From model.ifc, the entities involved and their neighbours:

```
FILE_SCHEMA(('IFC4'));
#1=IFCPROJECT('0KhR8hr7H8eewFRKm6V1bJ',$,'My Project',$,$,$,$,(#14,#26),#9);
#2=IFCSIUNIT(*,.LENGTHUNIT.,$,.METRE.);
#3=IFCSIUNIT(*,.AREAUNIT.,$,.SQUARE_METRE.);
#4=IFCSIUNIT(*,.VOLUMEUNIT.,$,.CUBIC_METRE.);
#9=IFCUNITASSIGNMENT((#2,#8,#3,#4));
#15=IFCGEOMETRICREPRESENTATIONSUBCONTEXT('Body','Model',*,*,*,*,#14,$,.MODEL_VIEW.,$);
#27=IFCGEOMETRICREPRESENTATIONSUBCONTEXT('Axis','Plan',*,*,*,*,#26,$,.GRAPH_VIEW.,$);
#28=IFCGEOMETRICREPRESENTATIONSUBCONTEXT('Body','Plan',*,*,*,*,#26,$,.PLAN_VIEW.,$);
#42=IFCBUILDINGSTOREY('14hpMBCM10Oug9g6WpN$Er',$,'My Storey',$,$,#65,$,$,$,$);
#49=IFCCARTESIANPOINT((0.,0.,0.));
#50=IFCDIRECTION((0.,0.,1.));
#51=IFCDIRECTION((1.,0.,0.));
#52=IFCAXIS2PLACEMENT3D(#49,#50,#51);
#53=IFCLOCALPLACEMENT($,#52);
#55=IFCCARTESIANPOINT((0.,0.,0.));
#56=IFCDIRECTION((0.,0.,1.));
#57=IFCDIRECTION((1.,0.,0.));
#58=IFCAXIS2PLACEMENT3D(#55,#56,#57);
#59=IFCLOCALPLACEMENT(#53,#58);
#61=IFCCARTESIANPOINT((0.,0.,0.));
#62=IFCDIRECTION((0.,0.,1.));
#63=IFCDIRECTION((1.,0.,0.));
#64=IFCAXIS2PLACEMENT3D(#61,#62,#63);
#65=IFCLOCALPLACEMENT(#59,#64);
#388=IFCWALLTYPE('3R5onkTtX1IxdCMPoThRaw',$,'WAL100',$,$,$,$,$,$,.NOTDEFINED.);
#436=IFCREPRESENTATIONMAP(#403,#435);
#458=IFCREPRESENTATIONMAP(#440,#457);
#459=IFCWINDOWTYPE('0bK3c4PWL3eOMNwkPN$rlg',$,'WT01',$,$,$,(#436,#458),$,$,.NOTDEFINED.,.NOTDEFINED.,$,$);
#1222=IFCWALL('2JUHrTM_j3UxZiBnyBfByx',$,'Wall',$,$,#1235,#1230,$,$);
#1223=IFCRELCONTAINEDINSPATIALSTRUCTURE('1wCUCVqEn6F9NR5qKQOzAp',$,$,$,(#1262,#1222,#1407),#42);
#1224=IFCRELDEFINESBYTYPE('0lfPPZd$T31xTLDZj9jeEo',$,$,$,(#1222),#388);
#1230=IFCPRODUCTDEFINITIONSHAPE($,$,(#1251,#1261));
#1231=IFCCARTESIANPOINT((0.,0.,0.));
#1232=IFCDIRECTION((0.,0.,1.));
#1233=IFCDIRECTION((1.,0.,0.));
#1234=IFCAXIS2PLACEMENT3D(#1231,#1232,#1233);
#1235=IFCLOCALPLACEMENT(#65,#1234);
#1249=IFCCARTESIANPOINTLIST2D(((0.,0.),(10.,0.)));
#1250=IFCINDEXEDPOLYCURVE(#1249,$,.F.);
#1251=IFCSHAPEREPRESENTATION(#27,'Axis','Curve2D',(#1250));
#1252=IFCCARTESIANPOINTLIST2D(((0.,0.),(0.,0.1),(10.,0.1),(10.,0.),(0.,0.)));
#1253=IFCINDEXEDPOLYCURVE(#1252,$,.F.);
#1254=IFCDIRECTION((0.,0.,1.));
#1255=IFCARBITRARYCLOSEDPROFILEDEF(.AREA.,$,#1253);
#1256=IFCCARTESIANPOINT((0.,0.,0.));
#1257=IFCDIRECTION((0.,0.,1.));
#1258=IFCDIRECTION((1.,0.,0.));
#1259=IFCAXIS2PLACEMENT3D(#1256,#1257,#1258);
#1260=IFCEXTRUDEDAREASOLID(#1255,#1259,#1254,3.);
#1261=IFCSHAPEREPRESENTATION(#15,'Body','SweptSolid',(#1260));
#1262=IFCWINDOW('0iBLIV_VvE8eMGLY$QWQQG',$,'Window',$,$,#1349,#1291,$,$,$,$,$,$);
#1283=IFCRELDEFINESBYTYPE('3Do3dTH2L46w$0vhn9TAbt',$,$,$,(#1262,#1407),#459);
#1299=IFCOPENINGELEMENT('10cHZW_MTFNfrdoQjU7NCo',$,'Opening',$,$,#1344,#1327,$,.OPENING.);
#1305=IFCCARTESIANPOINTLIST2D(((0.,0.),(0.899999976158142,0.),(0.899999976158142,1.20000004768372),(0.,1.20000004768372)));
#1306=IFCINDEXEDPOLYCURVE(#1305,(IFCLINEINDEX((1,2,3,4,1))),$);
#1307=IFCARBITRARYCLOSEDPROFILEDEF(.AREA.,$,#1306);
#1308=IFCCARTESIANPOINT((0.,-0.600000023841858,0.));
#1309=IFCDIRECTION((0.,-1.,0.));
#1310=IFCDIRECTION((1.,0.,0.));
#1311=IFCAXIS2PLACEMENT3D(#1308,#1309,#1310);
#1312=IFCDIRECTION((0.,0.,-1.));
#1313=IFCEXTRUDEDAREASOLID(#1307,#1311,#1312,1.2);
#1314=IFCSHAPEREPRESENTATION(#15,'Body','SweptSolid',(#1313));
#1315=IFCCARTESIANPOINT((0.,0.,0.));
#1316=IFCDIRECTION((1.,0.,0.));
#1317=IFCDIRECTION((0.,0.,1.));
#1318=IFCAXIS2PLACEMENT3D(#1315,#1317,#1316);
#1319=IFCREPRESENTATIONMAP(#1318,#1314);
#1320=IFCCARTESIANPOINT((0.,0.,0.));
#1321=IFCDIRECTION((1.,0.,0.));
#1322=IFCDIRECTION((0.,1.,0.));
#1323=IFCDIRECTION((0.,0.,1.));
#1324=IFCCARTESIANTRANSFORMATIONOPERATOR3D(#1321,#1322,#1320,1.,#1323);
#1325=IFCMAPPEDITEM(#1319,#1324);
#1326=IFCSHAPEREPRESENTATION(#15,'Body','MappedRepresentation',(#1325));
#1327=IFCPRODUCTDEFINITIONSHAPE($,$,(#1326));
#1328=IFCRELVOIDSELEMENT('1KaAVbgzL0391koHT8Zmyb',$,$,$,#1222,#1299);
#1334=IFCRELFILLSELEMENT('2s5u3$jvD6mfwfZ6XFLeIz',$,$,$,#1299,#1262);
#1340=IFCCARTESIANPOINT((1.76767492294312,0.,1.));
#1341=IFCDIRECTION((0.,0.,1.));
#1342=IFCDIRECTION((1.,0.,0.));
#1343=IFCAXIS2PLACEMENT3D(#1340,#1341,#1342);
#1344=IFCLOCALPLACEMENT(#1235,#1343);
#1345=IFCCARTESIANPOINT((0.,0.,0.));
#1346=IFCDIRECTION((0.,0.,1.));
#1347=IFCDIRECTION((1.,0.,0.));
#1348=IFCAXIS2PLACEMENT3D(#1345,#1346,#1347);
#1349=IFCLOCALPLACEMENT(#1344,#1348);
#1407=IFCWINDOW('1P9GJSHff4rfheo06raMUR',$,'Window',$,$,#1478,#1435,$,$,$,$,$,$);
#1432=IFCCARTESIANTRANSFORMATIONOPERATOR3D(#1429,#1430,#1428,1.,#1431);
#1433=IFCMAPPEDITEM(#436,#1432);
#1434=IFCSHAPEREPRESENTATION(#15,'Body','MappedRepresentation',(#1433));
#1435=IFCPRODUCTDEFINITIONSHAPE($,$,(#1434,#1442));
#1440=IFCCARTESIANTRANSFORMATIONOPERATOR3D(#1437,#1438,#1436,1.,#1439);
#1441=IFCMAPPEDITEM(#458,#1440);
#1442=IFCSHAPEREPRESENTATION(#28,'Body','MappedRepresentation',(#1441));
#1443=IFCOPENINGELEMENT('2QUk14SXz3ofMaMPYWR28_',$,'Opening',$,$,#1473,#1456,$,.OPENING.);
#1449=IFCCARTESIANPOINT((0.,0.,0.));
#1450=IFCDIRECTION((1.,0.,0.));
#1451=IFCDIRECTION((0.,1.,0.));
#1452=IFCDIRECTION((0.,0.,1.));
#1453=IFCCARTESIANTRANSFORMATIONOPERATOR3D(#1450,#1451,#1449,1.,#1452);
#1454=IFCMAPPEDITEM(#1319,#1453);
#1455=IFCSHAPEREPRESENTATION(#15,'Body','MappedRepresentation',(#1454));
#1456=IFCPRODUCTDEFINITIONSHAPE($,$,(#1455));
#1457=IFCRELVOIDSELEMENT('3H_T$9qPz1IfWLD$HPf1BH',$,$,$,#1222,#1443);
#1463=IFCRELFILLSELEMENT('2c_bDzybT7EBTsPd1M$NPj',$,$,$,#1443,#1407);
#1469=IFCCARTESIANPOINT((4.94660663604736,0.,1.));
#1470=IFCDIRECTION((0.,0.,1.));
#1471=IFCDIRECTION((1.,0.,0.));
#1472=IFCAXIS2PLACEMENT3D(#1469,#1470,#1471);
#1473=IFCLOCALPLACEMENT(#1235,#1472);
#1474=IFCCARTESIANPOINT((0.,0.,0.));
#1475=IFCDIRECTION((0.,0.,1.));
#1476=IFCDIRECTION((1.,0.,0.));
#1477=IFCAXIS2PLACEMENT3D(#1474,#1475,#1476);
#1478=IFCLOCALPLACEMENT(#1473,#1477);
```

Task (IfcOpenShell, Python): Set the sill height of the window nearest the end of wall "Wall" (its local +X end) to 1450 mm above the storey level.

```python
import numpy as np
import ifcopenshell
import ifcopenshell.api.geometry
import ifcopenshell.geom
import ifcopenshell.util.element
import ifcopenshell.util.placement
import ifcopenshell.util.shape
import ifcopenshell.util.unit

model = ifcopenshell.open("model.ifc")
unit_scale = ifcopenshell.util.unit.calculate_unit_scale(model)

window = model.by_guid("1P9GJSHff4rfheo06raMUR")
opening = window.FillsVoids[0].RelatingOpeningElement
storey = ifcopenshell.util.element.get_container(window, ifc_class="IfcBuildingStorey")
level = ifcopenshell.util.placement.get_local_placement(storey.ObjectPlacement)[2, 3]

# The opening's origin need not be at the sill, so measure its lowest point.
shape = ifcopenshell.geom.create_shape(ifcopenshell.geom.settings(), opening)
bottom = ifcopenshell.util.shape.get_shape_bottom_elevation(shape, shape.geometry) / unit_scale
dz = level + 1.45 - bottom

shift = np.array([0.0, 0.0, dz])
# The window is placed relative to its opening, so it follows when the opening moves.
matrix = ifcopenshell.util.placement.get_local_placement(opening.ObjectPlacement)
matrix[:3, 3] += shift
ifcopenshell.api.geometry.edit_object_placement(
    model, product=opening, matrix=matrix, is_si=False, should_transform_children=True
)

print(f"moved by {dz * unit_scale:+.3f} m")

model.write("model_v2.ifc")
```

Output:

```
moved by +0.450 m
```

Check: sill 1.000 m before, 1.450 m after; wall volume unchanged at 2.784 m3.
